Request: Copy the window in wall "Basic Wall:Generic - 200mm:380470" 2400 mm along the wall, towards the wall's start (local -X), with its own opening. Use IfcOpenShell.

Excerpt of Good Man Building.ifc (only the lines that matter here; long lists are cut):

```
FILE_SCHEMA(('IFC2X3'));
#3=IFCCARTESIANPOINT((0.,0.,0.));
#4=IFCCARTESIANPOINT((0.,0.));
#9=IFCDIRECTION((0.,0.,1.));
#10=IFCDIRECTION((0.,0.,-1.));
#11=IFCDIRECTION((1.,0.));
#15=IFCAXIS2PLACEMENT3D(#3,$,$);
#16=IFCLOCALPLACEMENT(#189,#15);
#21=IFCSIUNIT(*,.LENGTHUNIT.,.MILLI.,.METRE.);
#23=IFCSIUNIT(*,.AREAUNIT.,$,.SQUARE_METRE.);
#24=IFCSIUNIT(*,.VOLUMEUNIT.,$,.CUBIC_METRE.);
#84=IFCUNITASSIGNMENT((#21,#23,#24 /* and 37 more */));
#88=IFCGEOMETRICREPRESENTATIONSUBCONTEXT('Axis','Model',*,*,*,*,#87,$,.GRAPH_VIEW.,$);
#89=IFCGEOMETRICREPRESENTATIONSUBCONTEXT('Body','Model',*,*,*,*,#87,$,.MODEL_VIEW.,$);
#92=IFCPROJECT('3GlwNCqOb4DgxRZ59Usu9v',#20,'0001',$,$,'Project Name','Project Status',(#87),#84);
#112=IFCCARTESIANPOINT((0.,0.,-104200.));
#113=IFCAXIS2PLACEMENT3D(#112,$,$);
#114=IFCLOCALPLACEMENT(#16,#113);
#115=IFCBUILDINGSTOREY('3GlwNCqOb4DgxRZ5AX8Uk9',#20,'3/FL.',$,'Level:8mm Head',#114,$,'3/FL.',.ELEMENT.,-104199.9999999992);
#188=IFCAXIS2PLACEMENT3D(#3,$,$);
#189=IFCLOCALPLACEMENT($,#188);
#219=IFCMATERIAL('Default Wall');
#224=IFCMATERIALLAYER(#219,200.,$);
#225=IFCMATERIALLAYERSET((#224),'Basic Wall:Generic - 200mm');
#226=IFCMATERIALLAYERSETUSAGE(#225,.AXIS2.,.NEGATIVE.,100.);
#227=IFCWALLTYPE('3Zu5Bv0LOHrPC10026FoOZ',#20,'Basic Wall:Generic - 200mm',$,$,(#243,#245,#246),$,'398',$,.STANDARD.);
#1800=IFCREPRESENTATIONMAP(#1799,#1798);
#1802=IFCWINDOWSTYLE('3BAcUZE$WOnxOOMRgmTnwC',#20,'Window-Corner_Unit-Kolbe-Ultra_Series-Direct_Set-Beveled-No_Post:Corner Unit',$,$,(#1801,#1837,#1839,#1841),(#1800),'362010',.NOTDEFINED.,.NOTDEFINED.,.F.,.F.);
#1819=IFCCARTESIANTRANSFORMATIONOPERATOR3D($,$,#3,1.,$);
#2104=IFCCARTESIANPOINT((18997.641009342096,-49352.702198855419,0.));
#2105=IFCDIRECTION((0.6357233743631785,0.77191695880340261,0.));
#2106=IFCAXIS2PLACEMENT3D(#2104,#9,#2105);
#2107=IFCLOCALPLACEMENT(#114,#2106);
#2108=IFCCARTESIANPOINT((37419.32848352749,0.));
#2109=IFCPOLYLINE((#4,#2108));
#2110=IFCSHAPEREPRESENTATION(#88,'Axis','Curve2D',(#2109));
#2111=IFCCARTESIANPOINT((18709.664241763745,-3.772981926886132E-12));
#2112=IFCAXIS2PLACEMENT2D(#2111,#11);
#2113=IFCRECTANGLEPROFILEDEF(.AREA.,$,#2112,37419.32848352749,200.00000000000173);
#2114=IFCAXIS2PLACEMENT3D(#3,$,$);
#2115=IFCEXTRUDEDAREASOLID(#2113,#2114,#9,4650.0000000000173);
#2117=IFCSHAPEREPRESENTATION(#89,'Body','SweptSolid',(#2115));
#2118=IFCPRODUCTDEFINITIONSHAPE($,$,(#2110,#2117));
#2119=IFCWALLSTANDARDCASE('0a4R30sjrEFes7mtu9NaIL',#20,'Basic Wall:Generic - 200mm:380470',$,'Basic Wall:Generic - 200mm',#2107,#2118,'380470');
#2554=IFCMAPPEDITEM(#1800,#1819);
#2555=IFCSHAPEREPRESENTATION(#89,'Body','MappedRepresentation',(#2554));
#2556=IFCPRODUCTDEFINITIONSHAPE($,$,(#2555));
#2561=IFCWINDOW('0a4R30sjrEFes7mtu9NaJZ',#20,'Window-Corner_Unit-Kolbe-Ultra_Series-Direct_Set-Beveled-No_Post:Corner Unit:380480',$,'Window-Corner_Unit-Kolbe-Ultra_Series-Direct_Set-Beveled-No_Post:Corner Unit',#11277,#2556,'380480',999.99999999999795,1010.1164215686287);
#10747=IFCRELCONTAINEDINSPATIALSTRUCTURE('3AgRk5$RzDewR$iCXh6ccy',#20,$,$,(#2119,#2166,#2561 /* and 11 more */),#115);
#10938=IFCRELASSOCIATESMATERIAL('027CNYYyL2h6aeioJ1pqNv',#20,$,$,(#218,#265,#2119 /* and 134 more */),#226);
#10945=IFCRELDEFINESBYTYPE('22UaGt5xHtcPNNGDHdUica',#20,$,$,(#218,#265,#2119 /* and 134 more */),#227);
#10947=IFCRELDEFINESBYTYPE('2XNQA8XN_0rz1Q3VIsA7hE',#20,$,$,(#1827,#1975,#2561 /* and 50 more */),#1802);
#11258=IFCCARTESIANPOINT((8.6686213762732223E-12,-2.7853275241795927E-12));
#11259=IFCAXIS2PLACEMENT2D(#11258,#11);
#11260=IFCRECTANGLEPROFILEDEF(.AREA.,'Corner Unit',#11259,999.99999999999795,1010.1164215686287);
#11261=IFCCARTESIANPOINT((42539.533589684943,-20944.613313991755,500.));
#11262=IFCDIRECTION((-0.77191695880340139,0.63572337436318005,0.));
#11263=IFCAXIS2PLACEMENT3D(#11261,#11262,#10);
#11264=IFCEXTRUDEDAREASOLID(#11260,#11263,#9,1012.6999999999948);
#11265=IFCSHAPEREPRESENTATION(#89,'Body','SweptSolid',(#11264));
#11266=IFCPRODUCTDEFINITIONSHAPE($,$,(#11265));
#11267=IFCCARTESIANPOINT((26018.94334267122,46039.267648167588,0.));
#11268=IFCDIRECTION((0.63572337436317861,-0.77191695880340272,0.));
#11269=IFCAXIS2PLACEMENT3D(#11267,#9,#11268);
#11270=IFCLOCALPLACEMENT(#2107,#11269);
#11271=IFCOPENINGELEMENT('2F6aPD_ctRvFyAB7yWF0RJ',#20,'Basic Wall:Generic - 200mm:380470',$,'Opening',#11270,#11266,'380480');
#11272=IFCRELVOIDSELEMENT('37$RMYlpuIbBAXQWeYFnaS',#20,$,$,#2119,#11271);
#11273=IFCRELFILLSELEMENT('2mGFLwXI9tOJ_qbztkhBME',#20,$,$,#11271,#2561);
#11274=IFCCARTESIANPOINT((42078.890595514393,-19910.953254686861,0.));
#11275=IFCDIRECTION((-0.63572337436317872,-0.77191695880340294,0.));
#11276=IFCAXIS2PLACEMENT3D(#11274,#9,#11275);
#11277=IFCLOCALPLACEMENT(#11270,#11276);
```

```python
import ifcopenshell
import ifcopenshell.api.feature
import ifcopenshell.api.geometry
import ifcopenshell.api.root
import ifcopenshell.geom
import ifcopenshell.util.element
import ifcopenshell.util.placement
import ifcopenshell.util.shape
import ifcopenshell.util.unit

model = ifcopenshell.open("Good Man Building.ifc")
unit_scale = ifcopenshell.util.unit.calculate_unit_scale(model)
settings = ifcopenshell.geom.settings()


def volume(element):
    """Net volume in cubic metres, openings subtracted."""
    shape = ifcopenshell.geom.create_shape(settings, element)
    return ifcopenshell.util.shape.get_volume(shape.geometry)


def reuse_history(source, copy):
    """copy_class also copies each property set's owner history, people and application; keep the originals."""
    for rel in copy.IsDefinedBy:
        if rel.is_a("IfcRelDefinesByProperties") and (history := rel.RelatingPropertyDefinition.OwnerHistory):
            rel.RelatingPropertyDefinition.OwnerHistory = source.OwnerHistory
            ifcopenshell.util.element.remove_deep2(model, history)


window = model.by_id(2561)
opening = window.FillsVoids[0].RelatingOpeningElement
wall = opening.VoidsElements[0].RelatingBuildingElement
before = volume(wall)
shift = ifcopenshell.util.placement.get_local_placement(wall.ObjectPlacement)[:3, 0] * -2.4 / unit_scale

# copy_class copies the void relationship, type, container and properties, but no geometry.
new_opening = ifcopenshell.api.root.copy_class(model, product=opening)
new_opening.Representation = ifcopenshell.util.element.copy_deep(
    model, opening.Representation, exclude=["IfcGeometricRepresentationContext", "IfcRepresentationMap"]
)
new_opening.Name = "Basic Wall:Generic - 200mm"
new_opening.Tag = None
new_window = ifcopenshell.api.root.copy_class(model, product=window)
new_window.Representation = ifcopenshell.util.element.copy_deep(
    model, window.Representation, exclude=["IfcGeometricRepresentationContext", "IfcRepresentationMap"]
)
new_window.Name = "Window-Corner_Unit-Kolbe-Ultra_Series-Direct_Set-Beveled-No_Post:Corner Unit"
new_window.Tag = None
reuse_history(window, new_window)
fills = ifcopenshell.api.feature.add_filling(model, opening=new_opening, element=new_window)
fills.OwnerHistory = new_window.OwnerHistory  # required in IFC2X3

for old, new in ((opening, new_opening), (window, new_window)):
    matrix = ifcopenshell.util.placement.get_local_placement(old.ObjectPlacement)
    matrix[:3, 3] += shift
    ifcopenshell.api.geometry.edit_object_placement(model, product=new, matrix=matrix, is_si=False)

after = volume(wall)

print(f"wall volume {before:.3f} -> {after:.3f} m3")

model.write("Good Man Building_v2.ifc")
```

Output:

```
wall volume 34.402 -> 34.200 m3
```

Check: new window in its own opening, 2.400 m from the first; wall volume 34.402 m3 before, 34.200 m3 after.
